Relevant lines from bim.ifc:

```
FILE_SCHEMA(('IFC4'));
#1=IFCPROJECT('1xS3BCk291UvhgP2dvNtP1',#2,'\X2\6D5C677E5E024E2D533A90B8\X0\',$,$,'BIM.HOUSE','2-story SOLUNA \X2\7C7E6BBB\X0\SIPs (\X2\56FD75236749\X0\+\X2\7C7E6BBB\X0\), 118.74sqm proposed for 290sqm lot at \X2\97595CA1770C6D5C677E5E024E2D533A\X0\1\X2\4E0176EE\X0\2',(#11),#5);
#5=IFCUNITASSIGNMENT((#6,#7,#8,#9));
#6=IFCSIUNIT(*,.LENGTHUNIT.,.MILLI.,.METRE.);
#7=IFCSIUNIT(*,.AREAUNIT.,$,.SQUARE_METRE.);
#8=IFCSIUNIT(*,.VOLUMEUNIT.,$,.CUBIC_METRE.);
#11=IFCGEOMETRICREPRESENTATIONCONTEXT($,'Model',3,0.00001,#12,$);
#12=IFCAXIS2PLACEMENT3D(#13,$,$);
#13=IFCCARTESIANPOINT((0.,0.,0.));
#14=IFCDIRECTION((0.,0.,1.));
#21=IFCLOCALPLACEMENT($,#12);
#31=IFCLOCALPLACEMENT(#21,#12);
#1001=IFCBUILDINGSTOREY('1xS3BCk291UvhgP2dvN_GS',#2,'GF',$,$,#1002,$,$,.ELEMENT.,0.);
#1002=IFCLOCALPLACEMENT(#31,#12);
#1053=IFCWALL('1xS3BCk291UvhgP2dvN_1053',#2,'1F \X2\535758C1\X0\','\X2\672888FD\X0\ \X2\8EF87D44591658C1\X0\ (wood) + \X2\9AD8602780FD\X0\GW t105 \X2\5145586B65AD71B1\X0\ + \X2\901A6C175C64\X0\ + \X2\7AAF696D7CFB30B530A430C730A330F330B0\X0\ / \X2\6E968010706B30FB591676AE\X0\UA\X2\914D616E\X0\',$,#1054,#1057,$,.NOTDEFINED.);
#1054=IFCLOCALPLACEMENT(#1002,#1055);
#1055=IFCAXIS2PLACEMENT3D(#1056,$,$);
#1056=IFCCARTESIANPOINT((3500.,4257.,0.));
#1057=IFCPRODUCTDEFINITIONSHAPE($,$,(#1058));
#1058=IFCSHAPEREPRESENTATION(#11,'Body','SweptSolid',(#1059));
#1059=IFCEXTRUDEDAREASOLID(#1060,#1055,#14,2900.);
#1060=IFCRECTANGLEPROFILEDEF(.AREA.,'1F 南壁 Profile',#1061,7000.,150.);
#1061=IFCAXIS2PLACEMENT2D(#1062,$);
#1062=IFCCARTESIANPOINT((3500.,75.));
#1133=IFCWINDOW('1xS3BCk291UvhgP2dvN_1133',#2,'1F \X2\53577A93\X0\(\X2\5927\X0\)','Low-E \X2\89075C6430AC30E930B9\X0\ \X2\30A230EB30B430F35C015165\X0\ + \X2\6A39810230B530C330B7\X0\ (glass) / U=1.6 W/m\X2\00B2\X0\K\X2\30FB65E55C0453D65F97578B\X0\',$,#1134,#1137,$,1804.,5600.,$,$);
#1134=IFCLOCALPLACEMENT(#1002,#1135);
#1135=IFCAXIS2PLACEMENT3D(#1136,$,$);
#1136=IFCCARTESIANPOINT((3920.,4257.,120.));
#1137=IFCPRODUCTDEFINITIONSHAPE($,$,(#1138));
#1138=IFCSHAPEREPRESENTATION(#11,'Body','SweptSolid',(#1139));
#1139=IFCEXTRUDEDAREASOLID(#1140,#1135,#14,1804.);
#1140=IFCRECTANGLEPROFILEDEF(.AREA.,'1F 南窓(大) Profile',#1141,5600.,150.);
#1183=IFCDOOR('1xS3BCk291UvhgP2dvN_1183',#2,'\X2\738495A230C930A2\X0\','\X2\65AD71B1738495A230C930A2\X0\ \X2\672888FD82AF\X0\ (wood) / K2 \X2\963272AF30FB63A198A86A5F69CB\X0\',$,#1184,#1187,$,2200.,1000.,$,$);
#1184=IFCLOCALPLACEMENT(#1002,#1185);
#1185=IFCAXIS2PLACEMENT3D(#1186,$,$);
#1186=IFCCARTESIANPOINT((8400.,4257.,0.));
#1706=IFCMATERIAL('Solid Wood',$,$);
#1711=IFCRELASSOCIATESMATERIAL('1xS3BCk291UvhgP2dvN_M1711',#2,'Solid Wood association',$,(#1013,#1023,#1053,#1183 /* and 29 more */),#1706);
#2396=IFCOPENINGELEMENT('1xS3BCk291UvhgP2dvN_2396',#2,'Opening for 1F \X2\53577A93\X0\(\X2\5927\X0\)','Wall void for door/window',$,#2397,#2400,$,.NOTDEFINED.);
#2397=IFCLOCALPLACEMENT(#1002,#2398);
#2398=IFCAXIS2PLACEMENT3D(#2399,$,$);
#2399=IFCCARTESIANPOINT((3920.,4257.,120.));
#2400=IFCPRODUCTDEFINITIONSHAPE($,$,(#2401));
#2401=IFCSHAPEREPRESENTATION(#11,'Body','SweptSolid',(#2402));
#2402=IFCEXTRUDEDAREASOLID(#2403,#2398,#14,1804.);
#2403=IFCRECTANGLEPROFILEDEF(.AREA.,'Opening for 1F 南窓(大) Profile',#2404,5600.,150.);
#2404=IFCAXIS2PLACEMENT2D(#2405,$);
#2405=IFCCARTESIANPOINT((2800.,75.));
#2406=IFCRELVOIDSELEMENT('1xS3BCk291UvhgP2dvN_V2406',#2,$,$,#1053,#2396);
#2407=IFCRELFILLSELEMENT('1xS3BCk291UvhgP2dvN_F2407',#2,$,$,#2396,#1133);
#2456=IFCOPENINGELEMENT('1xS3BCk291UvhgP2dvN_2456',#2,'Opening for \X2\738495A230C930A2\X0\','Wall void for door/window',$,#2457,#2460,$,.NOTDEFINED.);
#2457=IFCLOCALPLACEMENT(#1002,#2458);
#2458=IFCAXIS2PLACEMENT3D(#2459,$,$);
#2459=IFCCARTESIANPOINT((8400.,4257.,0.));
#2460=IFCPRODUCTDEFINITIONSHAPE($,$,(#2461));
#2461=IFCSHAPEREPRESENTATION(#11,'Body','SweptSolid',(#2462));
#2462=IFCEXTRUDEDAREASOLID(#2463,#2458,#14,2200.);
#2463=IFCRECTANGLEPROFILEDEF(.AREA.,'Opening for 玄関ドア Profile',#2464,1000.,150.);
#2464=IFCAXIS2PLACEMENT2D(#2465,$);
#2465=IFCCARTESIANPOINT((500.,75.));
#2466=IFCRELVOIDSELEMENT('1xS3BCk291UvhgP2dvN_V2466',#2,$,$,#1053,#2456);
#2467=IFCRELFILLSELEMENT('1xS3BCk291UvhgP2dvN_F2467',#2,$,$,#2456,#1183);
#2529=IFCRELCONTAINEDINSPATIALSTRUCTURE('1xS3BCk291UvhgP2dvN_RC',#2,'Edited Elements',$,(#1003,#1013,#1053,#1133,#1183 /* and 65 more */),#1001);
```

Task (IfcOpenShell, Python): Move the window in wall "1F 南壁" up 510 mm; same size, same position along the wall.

```python
import numpy as np
import ifcopenshell
import ifcopenshell.api.geometry
import ifcopenshell.util.placement
import ifcopenshell.util.unit

model = ifcopenshell.open("bim.ifc")
unit_scale = ifcopenshell.util.unit.calculate_unit_scale(model)

window = model.by_id(1133)
opening = window.FillsVoids[0].RelatingOpeningElement
dz = 0.51 / unit_scale

shift = np.array([0.0, 0.0, dz])
# The window is not placed relative to its opening, so move both.
for product in (opening, window):
    matrix = ifcopenshell.util.placement.get_local_placement(product.ObjectPlacement)
    matrix[:3, 3] += shift
    ifcopenshell.api.geometry.edit_object_placement(model, product=product, matrix=matrix, is_si=False)

print(f"moved by {dz * unit_scale:+.3f} m")

model.write("bim_updated.ifc")
```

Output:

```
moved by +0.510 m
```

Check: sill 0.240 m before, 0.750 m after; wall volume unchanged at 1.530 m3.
